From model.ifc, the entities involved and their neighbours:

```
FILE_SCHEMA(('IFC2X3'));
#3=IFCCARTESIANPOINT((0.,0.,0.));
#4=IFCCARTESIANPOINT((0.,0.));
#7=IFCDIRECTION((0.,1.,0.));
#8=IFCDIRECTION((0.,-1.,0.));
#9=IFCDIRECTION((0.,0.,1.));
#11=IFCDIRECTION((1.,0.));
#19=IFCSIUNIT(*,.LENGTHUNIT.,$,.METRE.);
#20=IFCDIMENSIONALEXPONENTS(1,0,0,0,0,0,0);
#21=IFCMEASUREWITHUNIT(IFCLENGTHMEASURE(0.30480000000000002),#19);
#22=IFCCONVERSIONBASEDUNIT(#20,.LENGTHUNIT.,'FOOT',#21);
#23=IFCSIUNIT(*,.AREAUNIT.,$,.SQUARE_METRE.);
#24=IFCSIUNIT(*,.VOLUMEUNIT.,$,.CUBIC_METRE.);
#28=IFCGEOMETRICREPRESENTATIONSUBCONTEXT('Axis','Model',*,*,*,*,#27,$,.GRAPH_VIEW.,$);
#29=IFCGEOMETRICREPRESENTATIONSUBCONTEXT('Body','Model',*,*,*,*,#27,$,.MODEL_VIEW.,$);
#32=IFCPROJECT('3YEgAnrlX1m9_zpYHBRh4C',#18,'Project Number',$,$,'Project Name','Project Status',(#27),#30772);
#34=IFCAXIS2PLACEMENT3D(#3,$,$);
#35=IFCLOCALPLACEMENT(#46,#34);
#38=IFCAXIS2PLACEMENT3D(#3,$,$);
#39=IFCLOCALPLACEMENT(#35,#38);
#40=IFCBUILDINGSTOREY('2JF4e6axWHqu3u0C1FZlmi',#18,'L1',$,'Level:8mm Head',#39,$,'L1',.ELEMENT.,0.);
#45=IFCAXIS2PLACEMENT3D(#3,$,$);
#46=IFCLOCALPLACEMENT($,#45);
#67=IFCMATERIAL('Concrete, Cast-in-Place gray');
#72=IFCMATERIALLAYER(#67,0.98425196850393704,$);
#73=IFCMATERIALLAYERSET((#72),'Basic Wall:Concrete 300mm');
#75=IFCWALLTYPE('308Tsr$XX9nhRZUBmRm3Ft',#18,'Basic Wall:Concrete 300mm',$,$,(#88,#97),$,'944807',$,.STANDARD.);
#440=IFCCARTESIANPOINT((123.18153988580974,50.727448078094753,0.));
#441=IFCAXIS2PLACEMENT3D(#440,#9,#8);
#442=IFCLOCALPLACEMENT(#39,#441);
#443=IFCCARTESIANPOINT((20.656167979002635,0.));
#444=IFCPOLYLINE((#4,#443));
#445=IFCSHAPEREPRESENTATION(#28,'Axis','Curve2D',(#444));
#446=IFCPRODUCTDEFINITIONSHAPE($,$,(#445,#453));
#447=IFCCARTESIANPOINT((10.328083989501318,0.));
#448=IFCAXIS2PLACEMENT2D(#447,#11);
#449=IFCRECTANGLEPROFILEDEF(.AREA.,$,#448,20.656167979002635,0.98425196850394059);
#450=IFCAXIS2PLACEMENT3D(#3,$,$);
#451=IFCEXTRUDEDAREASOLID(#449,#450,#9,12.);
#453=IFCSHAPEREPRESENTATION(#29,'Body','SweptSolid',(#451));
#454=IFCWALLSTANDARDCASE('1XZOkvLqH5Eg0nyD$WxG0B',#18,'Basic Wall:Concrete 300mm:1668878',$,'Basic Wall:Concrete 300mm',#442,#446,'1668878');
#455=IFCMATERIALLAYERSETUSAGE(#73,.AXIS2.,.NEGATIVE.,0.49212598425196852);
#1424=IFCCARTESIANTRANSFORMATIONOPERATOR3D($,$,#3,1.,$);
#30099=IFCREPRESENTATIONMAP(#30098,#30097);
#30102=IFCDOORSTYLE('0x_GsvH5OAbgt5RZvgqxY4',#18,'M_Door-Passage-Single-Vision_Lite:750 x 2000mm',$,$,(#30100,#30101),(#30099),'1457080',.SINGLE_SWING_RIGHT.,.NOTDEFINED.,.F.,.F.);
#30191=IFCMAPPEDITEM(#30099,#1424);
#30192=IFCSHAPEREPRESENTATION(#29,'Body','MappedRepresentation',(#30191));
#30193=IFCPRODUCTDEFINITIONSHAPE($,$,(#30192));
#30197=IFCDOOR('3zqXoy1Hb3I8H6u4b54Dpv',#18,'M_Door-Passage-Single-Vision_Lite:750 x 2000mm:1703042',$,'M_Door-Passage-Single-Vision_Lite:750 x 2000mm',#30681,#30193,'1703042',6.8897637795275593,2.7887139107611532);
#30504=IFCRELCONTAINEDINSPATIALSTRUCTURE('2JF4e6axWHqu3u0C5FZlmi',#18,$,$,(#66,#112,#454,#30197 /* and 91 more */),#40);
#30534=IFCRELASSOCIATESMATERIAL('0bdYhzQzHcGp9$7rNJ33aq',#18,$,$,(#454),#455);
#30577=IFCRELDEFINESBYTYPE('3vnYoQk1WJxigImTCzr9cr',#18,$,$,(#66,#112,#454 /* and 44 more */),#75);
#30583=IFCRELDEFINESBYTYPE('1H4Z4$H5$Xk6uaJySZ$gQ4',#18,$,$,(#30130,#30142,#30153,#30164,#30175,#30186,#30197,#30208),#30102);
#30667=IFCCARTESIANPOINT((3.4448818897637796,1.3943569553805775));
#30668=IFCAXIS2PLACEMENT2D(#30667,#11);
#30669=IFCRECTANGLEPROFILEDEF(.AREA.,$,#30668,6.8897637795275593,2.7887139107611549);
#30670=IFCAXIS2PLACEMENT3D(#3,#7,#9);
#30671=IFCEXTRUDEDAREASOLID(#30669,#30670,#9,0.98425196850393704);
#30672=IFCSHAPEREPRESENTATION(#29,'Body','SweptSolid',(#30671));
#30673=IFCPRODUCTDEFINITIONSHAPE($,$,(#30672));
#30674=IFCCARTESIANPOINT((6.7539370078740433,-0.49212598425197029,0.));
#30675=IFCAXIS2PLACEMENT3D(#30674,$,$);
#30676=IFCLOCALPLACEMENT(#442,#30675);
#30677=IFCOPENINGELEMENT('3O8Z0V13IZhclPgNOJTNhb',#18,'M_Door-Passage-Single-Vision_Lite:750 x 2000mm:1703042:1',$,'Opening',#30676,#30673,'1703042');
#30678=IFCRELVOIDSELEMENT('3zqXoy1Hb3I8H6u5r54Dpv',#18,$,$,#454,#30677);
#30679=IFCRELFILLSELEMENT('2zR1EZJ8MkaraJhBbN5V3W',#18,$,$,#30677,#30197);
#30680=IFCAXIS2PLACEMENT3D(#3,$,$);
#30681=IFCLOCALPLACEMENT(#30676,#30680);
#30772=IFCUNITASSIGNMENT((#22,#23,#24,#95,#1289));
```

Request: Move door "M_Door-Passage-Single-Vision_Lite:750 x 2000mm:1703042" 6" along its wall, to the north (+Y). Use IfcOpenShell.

```python
import ifcopenshell
import ifcopenshell.api.geometry
import ifcopenshell.util.placement
import ifcopenshell.util.unit

model = ifcopenshell.open("model.ifc")
unit_scale = ifcopenshell.util.unit.calculate_unit_scale(model)

door = model.by_id(30197)
opening = door.FillsVoids[0].RelatingOpeningElement
wall = opening.VoidsElements[0].RelatingBuildingElement

wall_matrix = ifcopenshell.util.placement.get_local_placement(wall.ObjectPlacement)
shift = wall_matrix[:3, 0] * -6 * 0.0254 / unit_scale
before = ifcopenshell.util.placement.get_local_placement(door.ObjectPlacement)[:3, 3].copy()

# The door is placed relative to its opening, so it follows when the opening moves.
matrix = ifcopenshell.util.placement.get_local_placement(opening.ObjectPlacement)
matrix[:3, 3] += shift
ifcopenshell.api.geometry.edit_object_placement(
    model, product=opening, matrix=matrix, is_si=False, should_transform_children=True
)

after = ifcopenshell.util.placement.get_local_placement(door.ObjectPlacement)[:3, 3]
print("door moved by", (after - before).round(3) + 0.0)

model.write("model_v2.ifc")
```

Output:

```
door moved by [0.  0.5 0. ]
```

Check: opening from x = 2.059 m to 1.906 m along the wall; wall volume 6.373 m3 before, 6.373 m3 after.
